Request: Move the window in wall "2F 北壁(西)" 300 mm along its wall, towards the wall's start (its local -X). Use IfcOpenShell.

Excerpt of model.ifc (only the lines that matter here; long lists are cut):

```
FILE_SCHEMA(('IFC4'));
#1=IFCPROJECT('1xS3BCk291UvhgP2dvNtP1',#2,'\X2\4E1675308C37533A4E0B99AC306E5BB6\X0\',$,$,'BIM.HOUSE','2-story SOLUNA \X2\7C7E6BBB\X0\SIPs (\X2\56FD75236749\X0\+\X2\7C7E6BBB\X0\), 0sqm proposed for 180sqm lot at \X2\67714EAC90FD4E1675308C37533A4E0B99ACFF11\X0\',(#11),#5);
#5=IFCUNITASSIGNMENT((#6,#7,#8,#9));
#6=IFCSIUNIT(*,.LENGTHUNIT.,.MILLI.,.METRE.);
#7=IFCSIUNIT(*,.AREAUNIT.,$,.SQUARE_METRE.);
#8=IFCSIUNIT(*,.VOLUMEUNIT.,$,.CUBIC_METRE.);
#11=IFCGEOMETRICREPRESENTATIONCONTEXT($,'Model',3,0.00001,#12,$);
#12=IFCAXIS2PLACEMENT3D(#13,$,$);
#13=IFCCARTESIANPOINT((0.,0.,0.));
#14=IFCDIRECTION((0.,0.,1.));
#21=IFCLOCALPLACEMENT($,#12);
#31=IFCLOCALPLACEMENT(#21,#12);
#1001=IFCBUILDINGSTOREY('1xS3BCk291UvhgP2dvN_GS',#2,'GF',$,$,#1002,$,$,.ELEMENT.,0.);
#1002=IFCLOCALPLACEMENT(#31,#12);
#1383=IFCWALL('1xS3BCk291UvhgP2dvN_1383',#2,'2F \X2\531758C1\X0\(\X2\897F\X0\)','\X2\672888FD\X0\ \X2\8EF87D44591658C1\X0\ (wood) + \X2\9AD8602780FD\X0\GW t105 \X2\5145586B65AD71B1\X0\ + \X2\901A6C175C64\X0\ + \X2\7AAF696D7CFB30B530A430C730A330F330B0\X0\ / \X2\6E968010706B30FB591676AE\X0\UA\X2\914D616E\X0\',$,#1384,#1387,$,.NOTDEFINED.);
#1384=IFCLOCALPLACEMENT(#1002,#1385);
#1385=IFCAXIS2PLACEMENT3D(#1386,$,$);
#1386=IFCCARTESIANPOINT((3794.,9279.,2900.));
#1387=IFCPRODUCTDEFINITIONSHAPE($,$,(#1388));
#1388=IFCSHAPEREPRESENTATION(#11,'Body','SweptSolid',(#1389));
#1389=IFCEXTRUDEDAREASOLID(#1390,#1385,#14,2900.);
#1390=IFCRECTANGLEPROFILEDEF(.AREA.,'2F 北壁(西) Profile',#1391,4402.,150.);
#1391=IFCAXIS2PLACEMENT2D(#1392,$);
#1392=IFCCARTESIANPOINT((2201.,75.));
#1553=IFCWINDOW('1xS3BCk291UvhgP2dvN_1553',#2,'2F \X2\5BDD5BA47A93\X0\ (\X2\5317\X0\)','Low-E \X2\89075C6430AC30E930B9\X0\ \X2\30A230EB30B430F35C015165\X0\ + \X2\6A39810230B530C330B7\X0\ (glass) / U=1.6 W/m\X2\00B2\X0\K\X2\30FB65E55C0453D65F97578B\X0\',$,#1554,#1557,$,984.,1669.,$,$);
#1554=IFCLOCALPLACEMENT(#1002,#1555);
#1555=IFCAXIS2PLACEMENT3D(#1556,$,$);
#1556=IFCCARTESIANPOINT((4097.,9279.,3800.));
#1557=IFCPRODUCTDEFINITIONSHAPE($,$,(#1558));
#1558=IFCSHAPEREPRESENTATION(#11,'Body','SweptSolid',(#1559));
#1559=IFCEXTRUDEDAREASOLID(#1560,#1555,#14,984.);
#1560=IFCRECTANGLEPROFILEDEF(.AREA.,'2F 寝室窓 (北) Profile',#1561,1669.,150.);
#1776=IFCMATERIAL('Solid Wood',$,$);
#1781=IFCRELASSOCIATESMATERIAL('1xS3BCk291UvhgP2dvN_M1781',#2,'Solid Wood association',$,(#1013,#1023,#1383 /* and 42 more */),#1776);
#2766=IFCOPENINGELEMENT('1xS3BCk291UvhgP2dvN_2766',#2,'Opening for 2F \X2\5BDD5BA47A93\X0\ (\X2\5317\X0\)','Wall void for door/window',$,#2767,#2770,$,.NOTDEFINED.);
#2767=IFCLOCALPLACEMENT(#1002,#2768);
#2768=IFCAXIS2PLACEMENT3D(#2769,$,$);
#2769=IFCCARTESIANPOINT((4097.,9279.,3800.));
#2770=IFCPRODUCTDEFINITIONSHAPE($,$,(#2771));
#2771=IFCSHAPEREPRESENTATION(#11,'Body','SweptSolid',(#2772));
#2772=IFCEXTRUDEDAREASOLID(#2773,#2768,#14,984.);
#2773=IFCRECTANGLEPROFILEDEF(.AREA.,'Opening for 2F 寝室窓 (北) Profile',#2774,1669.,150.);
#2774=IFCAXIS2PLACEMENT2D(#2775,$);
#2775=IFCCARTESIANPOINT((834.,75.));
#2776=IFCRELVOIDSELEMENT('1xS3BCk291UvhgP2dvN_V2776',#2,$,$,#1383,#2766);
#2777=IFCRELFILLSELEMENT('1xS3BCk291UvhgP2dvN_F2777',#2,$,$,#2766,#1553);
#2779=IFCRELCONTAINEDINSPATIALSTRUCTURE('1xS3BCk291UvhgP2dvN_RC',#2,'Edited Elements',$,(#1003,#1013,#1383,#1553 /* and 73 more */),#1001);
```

```python
import ifcopenshell
import ifcopenshell.api.geometry
import ifcopenshell.util.placement
import ifcopenshell.util.unit

model = ifcopenshell.open("model.ifc")
unit_scale = ifcopenshell.util.unit.calculate_unit_scale(model)

window = model.by_guid("1xS3BCk291UvhgP2dvN_1553")
opening = window.FillsVoids[0].RelatingOpeningElement
wall = opening.VoidsElements[0].RelatingBuildingElement

wall_matrix = ifcopenshell.util.placement.get_local_placement(wall.ObjectPlacement)
shift = wall_matrix[:3, 0] * -0.3 / unit_scale
before = ifcopenshell.util.placement.get_local_placement(window.ObjectPlacement)[:3, 3].copy()

# The window is not placed relative to its opening, so move both.
for product in (opening, window):
    matrix = ifcopenshell.util.placement.get_local_placement(product.ObjectPlacement)
    matrix[:3, 3] += shift
    ifcopenshell.api.geometry.edit_object_placement(model, product=product, matrix=matrix, is_si=False)

after = ifcopenshell.util.placement.get_local_placement(window.ObjectPlacement)[:3, 3]
print("window moved by", (after - before).round(3) + 0.0)

model.write("model-out.ifc")
```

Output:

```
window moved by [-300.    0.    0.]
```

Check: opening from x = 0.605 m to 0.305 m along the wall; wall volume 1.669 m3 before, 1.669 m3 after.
